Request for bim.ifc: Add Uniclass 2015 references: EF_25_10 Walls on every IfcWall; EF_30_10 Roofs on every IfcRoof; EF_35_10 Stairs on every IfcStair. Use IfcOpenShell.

First a look at what the model holds.

```python
import ifcopenshell

model = ifcopenshell.open("bim.ifc")
print(model.schema)
print("classifications:", [c.Name for c in model.by_type("IfcClassification")])
for ifc_class in ("IfcDoor", "IfcRoof", "IfcStair", "IfcWall", "IfcWindow"):
    print(ifc_class, len(model.by_type(ifc_class)))
```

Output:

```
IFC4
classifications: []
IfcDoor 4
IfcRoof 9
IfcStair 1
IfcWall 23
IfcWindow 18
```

```python
import ifcopenshell
import ifcopenshell.api.classification

model = ifcopenshell.open("bim.ifc")

system = ifcopenshell.api.classification.add_classification(model, classification="Uniclass 2015")

codes = {
    "IfcWall": ("EF_25_10", "Walls"),
    "IfcRoof": ("EF_30_10", "Roofs"),
    "IfcStair": ("EF_35_10", "Stairs"),
}
for ifc_class, (code, name) in codes.items():
    products = model.by_type(ifc_class)
    ifcopenshell.api.classification.add_reference(
        model, products=products, classification=system, identification=code, name=name
    )
    print(code, len(products))

model.write("bim_rev.ifc")
```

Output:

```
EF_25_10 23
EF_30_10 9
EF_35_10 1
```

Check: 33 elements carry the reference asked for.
